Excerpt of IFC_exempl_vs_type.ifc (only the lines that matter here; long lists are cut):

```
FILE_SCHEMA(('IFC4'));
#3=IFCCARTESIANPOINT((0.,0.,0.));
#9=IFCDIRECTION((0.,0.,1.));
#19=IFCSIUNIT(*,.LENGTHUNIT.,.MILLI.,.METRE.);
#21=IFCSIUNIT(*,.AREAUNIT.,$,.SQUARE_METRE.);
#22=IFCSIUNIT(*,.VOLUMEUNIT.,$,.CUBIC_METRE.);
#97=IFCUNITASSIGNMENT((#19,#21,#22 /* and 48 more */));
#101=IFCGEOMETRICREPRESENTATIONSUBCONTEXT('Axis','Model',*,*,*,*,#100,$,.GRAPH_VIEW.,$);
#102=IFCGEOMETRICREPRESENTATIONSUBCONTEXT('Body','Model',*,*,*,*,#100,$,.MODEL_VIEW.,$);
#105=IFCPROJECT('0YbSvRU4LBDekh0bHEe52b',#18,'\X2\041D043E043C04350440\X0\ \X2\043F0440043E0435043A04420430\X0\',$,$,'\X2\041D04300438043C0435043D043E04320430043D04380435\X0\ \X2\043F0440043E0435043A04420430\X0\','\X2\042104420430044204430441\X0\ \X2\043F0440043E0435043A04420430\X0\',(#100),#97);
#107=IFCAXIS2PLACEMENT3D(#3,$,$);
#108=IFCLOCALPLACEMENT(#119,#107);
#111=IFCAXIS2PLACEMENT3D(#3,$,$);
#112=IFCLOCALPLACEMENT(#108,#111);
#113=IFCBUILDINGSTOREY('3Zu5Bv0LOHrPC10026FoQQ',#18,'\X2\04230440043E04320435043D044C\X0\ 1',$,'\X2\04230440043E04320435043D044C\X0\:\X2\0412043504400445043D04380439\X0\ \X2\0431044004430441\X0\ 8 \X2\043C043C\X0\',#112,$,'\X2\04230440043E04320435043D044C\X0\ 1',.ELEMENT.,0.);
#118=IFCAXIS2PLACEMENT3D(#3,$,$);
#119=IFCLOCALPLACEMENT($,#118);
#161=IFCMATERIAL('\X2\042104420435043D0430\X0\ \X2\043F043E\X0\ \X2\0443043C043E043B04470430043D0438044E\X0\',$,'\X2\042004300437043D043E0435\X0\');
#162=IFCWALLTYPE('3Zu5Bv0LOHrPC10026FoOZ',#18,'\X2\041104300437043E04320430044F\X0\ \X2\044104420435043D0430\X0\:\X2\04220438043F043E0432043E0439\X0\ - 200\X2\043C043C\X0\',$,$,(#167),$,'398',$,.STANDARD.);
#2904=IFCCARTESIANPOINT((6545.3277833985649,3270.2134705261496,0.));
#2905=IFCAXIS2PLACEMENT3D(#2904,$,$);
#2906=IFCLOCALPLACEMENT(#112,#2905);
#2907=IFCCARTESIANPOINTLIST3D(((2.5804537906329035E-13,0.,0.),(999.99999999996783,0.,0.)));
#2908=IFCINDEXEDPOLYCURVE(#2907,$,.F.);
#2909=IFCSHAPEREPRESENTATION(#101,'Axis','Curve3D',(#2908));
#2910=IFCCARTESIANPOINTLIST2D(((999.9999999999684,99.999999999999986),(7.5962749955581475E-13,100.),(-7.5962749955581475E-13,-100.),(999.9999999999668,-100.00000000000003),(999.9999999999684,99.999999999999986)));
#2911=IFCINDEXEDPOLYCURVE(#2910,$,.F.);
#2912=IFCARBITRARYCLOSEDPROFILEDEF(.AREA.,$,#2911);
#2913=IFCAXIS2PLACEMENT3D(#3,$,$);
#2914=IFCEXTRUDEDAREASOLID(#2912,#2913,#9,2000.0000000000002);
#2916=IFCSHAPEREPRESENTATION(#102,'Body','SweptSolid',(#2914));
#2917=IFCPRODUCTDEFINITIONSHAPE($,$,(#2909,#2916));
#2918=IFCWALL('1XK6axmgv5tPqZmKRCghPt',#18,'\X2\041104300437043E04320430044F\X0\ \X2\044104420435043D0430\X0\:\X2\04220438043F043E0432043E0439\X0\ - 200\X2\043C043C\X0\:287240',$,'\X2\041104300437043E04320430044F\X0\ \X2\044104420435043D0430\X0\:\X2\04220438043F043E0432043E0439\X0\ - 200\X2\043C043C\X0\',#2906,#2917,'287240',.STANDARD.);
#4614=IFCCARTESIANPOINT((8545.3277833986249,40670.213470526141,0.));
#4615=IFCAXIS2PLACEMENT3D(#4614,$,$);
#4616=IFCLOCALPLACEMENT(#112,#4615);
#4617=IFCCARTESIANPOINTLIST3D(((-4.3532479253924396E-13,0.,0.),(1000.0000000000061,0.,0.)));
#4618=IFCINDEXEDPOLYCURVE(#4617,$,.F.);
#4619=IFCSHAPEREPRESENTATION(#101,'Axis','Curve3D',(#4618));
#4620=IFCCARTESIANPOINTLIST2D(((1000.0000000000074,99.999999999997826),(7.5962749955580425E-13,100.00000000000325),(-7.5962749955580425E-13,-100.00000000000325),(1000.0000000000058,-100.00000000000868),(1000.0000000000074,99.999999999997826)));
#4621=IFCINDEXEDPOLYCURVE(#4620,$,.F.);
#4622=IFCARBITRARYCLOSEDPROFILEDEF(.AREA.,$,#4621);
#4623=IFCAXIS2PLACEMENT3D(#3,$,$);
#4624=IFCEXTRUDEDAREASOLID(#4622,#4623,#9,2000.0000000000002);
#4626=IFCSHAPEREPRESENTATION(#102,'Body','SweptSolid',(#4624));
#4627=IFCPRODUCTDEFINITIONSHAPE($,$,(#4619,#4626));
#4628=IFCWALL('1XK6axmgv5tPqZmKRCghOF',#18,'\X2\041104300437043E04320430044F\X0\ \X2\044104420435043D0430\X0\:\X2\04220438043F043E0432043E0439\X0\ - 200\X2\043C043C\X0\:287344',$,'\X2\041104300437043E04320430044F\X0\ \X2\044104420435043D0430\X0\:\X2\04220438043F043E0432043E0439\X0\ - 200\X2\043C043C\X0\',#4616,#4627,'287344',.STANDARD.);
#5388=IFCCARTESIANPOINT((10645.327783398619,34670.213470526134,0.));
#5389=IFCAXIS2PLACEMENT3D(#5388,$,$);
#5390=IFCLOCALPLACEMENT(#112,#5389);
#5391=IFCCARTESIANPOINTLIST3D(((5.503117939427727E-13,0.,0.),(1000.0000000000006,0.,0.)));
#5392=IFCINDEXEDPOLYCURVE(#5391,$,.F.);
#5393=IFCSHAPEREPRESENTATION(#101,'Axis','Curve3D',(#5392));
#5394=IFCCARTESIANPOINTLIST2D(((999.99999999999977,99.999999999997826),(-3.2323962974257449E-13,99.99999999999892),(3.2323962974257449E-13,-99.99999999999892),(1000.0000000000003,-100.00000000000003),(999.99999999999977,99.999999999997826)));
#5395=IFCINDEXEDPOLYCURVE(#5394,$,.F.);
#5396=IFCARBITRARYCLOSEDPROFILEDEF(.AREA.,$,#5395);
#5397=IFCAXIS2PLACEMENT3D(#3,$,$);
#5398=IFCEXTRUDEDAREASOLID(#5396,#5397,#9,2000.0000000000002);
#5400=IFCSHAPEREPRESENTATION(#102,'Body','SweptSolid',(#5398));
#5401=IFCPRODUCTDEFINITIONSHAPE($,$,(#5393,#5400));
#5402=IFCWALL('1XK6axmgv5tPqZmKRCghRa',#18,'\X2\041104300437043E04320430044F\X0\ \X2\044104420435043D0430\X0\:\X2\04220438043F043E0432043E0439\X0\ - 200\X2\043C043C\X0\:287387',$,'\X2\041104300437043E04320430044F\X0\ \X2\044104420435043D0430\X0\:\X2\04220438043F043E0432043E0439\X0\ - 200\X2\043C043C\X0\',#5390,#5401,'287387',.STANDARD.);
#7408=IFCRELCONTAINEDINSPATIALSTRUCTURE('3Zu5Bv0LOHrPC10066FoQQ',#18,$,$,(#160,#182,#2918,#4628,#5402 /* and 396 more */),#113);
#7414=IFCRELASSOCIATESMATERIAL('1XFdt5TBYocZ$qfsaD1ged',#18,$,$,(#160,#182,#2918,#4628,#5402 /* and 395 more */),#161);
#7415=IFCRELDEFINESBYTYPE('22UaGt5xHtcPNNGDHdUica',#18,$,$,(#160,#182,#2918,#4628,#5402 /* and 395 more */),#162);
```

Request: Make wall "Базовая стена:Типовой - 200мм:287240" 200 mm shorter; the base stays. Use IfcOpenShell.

```python
import ifcopenshell
import ifcopenshell.geom
import ifcopenshell.util.representation
import ifcopenshell.util.shape
import ifcopenshell.util.unit

model = ifcopenshell.open("IFC_exempl_vs_type.ifc")
unit_scale = ifcopenshell.util.unit.calculate_unit_scale(model)
settings = ifcopenshell.geom.settings()


def volume(element):
    """Net volume in cubic metres, openings subtracted."""
    shape = ifcopenshell.geom.create_shape(settings, element)
    return ifcopenshell.util.shape.get_volume(shape.geometry)


wall = model.by_guid("1XK6axmgv5tPqZmKRCghPt")
before = volume(wall)

body = ifcopenshell.util.representation.get_representation(wall, "Model", "Body")
solid = body.Items[0]
old_height = solid.Depth
solid.Depth -= 0.2 / unit_scale
after = volume(wall)

print(f"height {old_height:g} -> {solid.Depth:g}, volume {before:.3f} -> {after:.3f} m3")

model.write("IFC_exempl_vs_type_edited.ifc")
```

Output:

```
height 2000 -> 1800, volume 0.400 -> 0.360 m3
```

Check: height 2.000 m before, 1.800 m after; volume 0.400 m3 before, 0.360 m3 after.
